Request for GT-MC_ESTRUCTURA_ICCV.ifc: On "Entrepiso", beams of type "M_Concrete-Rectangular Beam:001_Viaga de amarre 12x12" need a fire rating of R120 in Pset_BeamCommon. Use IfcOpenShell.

First a look at what the model holds.

```python
import ifcopenshell
import ifcopenshell.util.element

model = ifcopenshell.open("GT-MC_ESTRUCTURA_ICCV.ifc")
print(model.schema)
storey = next(s for s in model.by_type("IfcBuildingStorey") if s.Name == "Entrepiso")
beams = [e for e in ifcopenshell.util.element.get_decomposition(storey) if e.is_a("IfcBeam")]
seen = {}
for e in beams:
    element_type = ifcopenshell.util.element.get_type(e)
    key = (element_type.Name if element_type != e and element_type else None, ifcopenshell.util.element.get_pset(e, "Pset_BeamCommon", "FireRating"))
    seen[key] = seen.get(key, 0) + 1
for (name, value), count in sorted(seen.items(), key=str):
    print(count, "x", name, "|", value)
```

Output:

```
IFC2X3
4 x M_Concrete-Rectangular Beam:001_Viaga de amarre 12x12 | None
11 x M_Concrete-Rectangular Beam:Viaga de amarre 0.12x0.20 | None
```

```python
import ifcopenshell
import ifcopenshell.api.pset
import ifcopenshell.util.element

model = ifcopenshell.open("GT-MC_ESTRUCTURA_ICCV.ifc")

storey = next(s for s in model.by_type("IfcBuildingStorey") if s.Name == "Entrepiso")
beams = [e for e in ifcopenshell.util.element.get_decomposition(storey) if e.is_a("IfcBeam")]

count = 0
for e in beams:
    element_type = ifcopenshell.util.element.get_type(e)
    if element_type in (None, e) or element_type.Name != "M_Concrete-Rectangular Beam:001_Viaga de amarre 12x12":
        continue
    # add_pset returns the element's existing set when there is one.
    pset = ifcopenshell.api.pset.add_pset(model, product=e, name="Pset_BeamCommon")
    ifcopenshell.api.pset.edit_pset(model, pset=pset, properties={"FireRating": "R120"})
    count += 1

print(count, "beams updated")

model.write("GT-MC_ESTRUCTURA_ICCV_v2.ifc")
```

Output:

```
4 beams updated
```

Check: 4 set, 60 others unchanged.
